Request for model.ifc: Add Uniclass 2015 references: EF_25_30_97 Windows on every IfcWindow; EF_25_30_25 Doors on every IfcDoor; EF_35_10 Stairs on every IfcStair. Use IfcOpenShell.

First a look at what the model holds.

```python
import ifcopenshell

model = ifcopenshell.open("model.ifc")
print(model.schema)
print("classifications:", [c.Name for c in model.by_type("IfcClassification")])
for ifc_class in ("IfcDoor", "IfcRoof", "IfcStair", "IfcWall", "IfcWindow"):
    print(ifc_class, len(model.by_type(ifc_class)))
```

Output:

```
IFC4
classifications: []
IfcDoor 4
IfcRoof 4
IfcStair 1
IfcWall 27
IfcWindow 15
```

```python
import ifcopenshell
import ifcopenshell.api.classification

model = ifcopenshell.open("model.ifc")

system = ifcopenshell.api.classification.add_classification(model, classification="Uniclass 2015")

codes = {
    "IfcWindow": ("EF_25_30_97", "Windows"),
    "IfcDoor": ("EF_25_30_25", "Doors"),
    "IfcStair": ("EF_35_10", "Stairs"),
}
for ifc_class, (code, name) in codes.items():
    products = model.by_type(ifc_class)
    ifcopenshell.api.classification.add_reference(
        model, products=products, classification=system, identification=code, name=name
    )
    print(code, len(products))

model.write("model_v2.ifc")
```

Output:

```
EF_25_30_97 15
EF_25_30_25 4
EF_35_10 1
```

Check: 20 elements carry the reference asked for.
